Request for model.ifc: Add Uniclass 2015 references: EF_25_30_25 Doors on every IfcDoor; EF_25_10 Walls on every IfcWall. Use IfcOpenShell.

First a look at what the model holds.

```python
import ifcopenshell

model = ifcopenshell.open("model.ifc")
print(model.schema)
print("classifications:", [c.Name for c in model.by_type("IfcClassification")])
for ifc_class in ("IfcDoor", "IfcRoof", "IfcStair", "IfcWall", "IfcWindow"):
    print(ifc_class, len(model.by_type(ifc_class)))
```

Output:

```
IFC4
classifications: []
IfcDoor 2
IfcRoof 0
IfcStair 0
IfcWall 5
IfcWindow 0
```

```python
import ifcopenshell
import ifcopenshell.api.classification

model = ifcopenshell.open("model.ifc")

system = ifcopenshell.api.classification.add_classification(model, classification="Uniclass 2015")

codes = {
    "IfcDoor": ("EF_25_30_25", "Doors"),
    "IfcWall": ("EF_25_10", "Walls"),
}
for ifc_class, (code, name) in codes.items():
    products = model.by_type(ifc_class)
    ifcopenshell.api.classification.add_reference(
        model, products=products, classification=system, identification=code, name=name
    )
    print(code, len(products))

model.write("model_v2.ifc")
```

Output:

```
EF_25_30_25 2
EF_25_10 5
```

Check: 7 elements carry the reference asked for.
